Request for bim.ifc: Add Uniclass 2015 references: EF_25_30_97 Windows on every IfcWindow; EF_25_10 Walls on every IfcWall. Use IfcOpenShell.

First a look at what the model holds.

```python
import ifcopenshell

model = ifcopenshell.open("bim.ifc")
print(model.schema)
print("classifications:", [c.Name for c in model.by_type("IfcClassification")])
for ifc_class in ("IfcDoor", "IfcRoof", "IfcStair", "IfcWall", "IfcWindow"):
    print(ifc_class, len(model.by_type(ifc_class)))
```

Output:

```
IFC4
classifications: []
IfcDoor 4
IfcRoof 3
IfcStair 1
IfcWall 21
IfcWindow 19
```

```python
import ifcopenshell
import ifcopenshell.api.classification

model = ifcopenshell.open("bim.ifc")

system = ifcopenshell.api.classification.add_classification(model, classification="Uniclass 2015")

codes = {
    "IfcWindow": ("EF_25_30_97", "Windows"),
    "IfcWall": ("EF_25_10", "Walls"),
}
for ifc_class, (code, name) in codes.items():
    products = model.by_type(ifc_class)
    ifcopenshell.api.classification.add_reference(
        model, products=products, classification=system, identification=code, name=name
    )
    print(code, len(products))

model.write("bim_v2.ifc")
```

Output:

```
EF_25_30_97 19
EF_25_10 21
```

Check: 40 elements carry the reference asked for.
